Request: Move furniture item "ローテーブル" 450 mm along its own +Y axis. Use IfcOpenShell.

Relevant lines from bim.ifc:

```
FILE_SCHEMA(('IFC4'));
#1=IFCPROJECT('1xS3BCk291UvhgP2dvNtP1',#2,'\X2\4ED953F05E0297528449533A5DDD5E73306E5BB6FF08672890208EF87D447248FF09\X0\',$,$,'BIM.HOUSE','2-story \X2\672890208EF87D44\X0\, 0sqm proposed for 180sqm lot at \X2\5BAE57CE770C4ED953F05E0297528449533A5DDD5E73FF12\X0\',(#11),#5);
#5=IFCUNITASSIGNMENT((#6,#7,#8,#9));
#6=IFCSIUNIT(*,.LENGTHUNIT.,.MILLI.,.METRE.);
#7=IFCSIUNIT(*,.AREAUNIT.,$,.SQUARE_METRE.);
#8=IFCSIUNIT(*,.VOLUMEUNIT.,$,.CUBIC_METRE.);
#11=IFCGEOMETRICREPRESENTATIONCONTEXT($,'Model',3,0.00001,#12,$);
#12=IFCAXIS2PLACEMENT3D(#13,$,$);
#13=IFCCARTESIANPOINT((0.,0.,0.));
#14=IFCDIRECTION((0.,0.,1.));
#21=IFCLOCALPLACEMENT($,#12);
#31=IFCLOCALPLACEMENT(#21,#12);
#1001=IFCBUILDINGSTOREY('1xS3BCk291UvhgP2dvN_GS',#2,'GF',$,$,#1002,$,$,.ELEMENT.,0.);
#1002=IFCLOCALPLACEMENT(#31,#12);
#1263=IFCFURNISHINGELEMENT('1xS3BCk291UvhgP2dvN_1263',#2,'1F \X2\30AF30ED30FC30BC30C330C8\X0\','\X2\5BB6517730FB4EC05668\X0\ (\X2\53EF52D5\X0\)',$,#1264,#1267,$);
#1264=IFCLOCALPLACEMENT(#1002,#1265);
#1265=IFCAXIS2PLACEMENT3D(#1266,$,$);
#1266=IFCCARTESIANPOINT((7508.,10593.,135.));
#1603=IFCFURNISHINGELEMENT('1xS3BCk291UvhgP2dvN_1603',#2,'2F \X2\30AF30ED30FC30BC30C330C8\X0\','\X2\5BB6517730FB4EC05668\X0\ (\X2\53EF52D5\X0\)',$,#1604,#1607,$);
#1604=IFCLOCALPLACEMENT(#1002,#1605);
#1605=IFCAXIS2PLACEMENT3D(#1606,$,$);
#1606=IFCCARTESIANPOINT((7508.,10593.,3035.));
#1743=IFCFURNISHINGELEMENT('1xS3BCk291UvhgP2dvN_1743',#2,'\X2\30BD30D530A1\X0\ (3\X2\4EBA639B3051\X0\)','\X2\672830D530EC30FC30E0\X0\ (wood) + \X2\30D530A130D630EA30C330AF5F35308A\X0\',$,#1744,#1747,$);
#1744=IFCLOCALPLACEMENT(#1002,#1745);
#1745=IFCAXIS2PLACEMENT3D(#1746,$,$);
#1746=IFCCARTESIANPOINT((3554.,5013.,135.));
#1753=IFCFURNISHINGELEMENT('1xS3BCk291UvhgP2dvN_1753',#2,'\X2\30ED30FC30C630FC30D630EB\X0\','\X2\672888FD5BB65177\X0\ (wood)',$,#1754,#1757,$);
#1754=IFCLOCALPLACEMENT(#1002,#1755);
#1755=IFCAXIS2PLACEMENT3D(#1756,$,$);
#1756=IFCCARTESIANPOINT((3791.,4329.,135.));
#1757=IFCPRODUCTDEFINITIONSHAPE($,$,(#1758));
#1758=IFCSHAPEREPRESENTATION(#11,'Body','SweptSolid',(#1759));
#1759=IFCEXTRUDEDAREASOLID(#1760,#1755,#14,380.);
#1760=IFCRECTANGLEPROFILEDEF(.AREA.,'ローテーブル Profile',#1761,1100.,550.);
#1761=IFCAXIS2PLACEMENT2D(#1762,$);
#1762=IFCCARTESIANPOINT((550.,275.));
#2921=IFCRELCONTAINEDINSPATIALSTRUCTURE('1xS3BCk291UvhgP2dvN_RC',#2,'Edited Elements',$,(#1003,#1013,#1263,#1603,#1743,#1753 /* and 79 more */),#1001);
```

```python
import ifcopenshell
import ifcopenshell.api.geometry
import ifcopenshell.util.placement

model = ifcopenshell.open("bim.ifc")

item = model.by_guid("1xS3BCk291UvhgP2dvN_1753")
matrix = ifcopenshell.util.placement.get_local_placement(item.ObjectPlacement)
matrix[:3, 3] += matrix[:3, 1] * 450.0
ifcopenshell.api.geometry.edit_object_placement(model, product=item, matrix=matrix, is_si=False)

print(ifcopenshell.util.placement.get_local_placement(item.ObjectPlacement).round(3) + 0.0)

model.write("bim_edited.ifc")
```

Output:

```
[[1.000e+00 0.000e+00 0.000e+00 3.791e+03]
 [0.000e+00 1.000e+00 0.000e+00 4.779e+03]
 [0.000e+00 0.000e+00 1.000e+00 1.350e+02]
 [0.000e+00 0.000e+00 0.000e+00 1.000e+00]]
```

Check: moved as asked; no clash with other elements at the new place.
